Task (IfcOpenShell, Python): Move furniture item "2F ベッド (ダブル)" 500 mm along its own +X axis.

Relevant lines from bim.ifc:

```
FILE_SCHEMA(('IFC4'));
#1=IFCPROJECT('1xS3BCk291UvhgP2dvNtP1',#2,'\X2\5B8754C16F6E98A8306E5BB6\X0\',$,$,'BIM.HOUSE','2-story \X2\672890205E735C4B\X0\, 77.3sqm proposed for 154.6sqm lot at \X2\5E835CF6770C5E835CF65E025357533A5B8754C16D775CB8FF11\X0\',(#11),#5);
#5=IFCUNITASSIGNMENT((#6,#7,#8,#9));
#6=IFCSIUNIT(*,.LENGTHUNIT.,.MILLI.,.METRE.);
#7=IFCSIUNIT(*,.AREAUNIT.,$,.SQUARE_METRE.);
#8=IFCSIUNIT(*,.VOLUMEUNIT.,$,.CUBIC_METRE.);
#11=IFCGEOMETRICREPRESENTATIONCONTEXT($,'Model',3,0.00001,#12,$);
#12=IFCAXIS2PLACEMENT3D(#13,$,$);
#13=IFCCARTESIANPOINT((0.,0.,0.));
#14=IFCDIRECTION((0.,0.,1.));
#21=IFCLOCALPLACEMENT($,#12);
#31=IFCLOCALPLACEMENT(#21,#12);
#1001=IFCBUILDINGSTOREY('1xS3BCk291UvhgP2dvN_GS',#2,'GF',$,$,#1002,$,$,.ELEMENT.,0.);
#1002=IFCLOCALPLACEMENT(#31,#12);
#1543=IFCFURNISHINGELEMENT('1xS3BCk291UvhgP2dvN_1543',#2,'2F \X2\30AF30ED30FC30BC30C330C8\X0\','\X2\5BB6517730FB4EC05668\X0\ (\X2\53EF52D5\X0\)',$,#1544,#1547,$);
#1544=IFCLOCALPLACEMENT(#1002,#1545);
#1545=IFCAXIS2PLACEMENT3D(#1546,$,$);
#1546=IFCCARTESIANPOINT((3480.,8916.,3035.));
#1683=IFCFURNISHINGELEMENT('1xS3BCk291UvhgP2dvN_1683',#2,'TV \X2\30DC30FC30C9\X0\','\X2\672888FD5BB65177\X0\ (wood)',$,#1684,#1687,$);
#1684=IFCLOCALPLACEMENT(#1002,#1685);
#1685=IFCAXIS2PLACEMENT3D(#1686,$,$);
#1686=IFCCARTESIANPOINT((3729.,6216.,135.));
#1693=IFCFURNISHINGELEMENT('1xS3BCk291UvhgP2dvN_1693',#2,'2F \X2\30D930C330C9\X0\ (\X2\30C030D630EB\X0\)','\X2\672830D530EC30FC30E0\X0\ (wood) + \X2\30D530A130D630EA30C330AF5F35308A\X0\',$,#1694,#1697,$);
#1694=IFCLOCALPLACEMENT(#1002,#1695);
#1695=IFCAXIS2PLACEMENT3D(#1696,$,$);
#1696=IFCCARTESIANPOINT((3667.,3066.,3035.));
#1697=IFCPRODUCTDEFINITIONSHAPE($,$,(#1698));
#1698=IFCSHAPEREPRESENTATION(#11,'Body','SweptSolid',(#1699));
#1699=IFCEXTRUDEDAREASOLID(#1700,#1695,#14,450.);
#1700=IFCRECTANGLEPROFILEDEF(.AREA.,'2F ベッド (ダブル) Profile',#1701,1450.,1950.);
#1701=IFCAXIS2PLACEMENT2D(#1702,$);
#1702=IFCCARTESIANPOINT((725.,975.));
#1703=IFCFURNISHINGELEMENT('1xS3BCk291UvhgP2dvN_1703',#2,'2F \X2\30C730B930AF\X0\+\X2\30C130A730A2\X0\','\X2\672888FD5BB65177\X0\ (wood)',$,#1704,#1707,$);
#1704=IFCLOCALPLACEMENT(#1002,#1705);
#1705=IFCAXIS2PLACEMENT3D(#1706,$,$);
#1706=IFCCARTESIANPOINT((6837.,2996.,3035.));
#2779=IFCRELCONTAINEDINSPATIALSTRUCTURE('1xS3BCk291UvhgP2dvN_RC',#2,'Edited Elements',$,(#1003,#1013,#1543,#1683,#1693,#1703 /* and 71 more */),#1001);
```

```python
import ifcopenshell
import ifcopenshell.api.geometry
import ifcopenshell.util.placement
import ifcopenshell.util.unit

model = ifcopenshell.open("bim.ifc")
unit_scale = ifcopenshell.util.unit.calculate_unit_scale(model)

item = model.by_id(1693)
matrix = ifcopenshell.util.placement.get_local_placement(item.ObjectPlacement)
matrix[:3, 3] += matrix[:3, 0] * 0.5 / unit_scale
ifcopenshell.api.geometry.edit_object_placement(model, product=item, matrix=matrix, is_si=False)

print(ifcopenshell.util.placement.get_local_placement(item.ObjectPlacement).round(3) + 0.0)

model.write("bim_v2.ifc")
```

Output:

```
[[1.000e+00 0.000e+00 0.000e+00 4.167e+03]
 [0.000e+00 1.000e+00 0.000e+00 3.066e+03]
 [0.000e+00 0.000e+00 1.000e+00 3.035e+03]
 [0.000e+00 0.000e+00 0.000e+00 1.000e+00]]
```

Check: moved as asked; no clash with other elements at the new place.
